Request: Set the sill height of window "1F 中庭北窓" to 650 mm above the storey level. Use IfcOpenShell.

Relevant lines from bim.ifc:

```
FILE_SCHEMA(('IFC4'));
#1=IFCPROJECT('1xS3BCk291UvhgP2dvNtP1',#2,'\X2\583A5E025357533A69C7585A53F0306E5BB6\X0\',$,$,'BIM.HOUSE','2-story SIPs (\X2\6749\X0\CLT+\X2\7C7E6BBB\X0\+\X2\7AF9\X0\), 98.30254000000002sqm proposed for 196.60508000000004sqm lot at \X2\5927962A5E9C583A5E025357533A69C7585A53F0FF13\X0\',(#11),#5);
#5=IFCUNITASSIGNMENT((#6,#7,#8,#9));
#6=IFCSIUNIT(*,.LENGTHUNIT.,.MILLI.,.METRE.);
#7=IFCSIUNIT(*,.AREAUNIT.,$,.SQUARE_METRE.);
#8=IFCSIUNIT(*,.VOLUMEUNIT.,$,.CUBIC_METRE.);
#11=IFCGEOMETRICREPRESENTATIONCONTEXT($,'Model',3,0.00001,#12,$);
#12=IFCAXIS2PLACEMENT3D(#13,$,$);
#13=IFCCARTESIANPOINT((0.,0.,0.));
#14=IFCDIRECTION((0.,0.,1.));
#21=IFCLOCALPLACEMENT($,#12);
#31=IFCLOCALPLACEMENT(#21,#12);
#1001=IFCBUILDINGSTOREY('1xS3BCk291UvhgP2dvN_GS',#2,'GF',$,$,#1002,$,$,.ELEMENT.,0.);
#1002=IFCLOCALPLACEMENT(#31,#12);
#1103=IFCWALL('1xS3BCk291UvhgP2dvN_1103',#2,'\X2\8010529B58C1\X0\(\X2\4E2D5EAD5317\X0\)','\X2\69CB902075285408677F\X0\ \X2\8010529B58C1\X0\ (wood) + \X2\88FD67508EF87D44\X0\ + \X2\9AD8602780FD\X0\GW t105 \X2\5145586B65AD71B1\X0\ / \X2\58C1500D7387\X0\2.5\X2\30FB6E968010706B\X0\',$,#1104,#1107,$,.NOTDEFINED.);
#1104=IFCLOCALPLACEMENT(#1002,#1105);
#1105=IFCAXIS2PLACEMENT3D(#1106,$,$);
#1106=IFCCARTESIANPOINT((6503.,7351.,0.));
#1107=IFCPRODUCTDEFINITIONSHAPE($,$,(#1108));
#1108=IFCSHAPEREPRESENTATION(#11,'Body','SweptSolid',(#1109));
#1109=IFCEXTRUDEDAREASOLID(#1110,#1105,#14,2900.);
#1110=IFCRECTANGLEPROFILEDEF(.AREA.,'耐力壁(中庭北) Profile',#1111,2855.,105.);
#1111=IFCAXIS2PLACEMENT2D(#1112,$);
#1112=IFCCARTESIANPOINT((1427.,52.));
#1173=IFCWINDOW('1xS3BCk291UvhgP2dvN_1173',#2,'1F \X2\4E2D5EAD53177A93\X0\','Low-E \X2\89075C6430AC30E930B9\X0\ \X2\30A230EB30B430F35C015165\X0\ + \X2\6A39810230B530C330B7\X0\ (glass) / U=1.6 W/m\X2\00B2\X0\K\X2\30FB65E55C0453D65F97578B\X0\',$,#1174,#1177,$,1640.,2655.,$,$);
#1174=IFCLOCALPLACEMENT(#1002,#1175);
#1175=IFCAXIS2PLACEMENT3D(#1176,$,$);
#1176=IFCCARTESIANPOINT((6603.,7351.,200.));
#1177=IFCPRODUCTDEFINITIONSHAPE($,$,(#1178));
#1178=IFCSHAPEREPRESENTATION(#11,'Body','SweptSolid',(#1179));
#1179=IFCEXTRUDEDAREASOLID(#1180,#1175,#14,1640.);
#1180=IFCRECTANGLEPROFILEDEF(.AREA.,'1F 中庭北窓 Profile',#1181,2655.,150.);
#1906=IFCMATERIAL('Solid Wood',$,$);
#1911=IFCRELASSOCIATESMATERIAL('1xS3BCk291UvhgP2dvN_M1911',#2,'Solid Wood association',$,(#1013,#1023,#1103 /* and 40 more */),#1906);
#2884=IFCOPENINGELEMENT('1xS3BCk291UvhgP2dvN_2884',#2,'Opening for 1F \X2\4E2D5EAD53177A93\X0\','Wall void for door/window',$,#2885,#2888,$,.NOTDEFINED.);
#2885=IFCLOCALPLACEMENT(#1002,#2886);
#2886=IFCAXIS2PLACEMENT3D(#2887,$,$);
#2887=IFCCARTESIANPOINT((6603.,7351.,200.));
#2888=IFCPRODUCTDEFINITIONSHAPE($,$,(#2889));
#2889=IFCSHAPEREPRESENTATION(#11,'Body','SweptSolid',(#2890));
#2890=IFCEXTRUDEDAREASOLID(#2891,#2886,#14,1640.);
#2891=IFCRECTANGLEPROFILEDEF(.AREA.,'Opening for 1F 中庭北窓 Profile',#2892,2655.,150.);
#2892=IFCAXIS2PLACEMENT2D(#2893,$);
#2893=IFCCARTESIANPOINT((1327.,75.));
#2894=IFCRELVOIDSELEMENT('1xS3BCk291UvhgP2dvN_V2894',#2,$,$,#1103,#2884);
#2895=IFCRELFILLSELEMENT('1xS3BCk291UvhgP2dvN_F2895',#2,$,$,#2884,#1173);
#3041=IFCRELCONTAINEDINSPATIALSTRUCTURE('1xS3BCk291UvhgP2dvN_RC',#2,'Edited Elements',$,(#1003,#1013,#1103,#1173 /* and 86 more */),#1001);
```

```python
import numpy as np
import ifcopenshell
import ifcopenshell.api.geometry
import ifcopenshell.geom
import ifcopenshell.util.element
import ifcopenshell.util.placement
import ifcopenshell.util.shape
import ifcopenshell.util.unit

model = ifcopenshell.open("bim.ifc")
unit_scale = ifcopenshell.util.unit.calculate_unit_scale(model)

window = model.by_guid("1xS3BCk291UvhgP2dvN_1173")
opening = window.FillsVoids[0].RelatingOpeningElement
storey = ifcopenshell.util.element.get_container(window, ifc_class="IfcBuildingStorey")
level = ifcopenshell.util.placement.get_local_placement(storey.ObjectPlacement)[2, 3]

# The opening's origin need not be at the sill, so measure its lowest point.
shape = ifcopenshell.geom.create_shape(ifcopenshell.geom.settings(), opening)
bottom = ifcopenshell.util.shape.get_shape_bottom_elevation(shape, shape.geometry) / unit_scale
dz = level + 650.0 - bottom

shift = np.array([0.0, 0.0, dz])
# The window is not placed relative to its opening, so move both.
for product in (opening, window):
    matrix = ifcopenshell.util.placement.get_local_placement(product.ObjectPlacement)
    matrix[:3, 3] += shift
    ifcopenshell.api.geometry.edit_object_placement(model, product=product, matrix=matrix, is_si=False)

print(f"moved by {dz * unit_scale:+.3f} m")

model.write("bim-out.ifc")
```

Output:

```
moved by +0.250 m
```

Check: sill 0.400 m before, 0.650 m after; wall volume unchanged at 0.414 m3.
